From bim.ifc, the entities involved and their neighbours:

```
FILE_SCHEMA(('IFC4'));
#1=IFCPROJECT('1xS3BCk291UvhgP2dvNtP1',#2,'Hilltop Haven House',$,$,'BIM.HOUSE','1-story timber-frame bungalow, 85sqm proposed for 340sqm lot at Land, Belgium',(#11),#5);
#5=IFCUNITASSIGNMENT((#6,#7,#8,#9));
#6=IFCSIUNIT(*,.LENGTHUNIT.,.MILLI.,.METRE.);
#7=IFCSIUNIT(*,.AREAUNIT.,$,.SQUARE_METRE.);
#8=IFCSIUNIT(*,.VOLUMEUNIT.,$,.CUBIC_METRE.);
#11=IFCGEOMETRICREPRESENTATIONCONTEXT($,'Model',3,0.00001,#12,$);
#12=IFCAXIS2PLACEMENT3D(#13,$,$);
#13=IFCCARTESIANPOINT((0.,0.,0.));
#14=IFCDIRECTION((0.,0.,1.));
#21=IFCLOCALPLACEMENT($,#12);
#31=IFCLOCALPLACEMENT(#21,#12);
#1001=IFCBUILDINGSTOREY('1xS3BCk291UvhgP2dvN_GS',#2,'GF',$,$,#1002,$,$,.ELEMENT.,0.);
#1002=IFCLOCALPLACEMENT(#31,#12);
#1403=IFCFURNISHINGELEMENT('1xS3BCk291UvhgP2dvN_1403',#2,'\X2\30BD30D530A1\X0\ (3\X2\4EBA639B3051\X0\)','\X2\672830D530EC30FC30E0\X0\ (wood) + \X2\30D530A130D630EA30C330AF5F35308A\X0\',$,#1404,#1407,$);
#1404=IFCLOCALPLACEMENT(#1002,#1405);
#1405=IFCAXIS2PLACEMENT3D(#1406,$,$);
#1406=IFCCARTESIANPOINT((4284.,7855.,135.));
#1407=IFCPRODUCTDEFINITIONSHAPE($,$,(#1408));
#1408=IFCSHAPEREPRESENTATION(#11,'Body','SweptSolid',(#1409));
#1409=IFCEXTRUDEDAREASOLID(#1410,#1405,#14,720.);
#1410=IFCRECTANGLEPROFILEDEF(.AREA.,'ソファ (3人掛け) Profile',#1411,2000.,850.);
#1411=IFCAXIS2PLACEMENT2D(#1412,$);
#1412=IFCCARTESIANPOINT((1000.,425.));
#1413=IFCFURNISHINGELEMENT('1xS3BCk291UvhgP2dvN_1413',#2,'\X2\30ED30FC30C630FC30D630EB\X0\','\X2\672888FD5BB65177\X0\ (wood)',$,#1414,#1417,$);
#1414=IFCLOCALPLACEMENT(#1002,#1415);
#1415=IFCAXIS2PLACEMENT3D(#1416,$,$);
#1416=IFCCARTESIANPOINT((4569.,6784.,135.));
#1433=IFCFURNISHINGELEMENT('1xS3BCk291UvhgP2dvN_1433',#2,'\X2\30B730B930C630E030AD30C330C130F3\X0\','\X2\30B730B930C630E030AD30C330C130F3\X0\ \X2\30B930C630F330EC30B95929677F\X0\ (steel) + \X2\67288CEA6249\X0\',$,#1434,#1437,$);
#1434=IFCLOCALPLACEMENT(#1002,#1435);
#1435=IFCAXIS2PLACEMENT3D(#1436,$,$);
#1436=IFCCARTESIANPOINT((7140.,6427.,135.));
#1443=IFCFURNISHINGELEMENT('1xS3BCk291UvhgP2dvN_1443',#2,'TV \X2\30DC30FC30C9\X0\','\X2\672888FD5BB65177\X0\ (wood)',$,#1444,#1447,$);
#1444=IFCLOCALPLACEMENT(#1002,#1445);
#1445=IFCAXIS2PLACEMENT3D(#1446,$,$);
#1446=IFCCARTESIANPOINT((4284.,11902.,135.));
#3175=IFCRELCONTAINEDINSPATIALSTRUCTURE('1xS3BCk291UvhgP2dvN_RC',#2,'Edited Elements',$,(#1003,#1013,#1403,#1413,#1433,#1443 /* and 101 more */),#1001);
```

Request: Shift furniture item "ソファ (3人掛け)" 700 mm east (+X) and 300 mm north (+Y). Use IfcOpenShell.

```python
import ifcopenshell
import ifcopenshell.api.geometry
import ifcopenshell.util.placement

model = ifcopenshell.open("bim.ifc")

item = model.by_guid("1xS3BCk291UvhgP2dvN_1403")
matrix = ifcopenshell.util.placement.get_local_placement(item.ObjectPlacement)
matrix[0, 3] += 700.0
matrix[1, 3] += 300.0
ifcopenshell.api.geometry.edit_object_placement(model, product=item, matrix=matrix, is_si=False)

print(ifcopenshell.util.placement.get_local_placement(item.ObjectPlacement).round(3) + 0.0)

model.write("bim_rev.ifc")
```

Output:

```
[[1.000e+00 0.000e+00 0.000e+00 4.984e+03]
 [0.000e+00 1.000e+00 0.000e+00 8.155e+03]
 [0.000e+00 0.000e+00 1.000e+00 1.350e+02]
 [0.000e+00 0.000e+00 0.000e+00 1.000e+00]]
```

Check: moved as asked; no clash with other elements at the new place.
